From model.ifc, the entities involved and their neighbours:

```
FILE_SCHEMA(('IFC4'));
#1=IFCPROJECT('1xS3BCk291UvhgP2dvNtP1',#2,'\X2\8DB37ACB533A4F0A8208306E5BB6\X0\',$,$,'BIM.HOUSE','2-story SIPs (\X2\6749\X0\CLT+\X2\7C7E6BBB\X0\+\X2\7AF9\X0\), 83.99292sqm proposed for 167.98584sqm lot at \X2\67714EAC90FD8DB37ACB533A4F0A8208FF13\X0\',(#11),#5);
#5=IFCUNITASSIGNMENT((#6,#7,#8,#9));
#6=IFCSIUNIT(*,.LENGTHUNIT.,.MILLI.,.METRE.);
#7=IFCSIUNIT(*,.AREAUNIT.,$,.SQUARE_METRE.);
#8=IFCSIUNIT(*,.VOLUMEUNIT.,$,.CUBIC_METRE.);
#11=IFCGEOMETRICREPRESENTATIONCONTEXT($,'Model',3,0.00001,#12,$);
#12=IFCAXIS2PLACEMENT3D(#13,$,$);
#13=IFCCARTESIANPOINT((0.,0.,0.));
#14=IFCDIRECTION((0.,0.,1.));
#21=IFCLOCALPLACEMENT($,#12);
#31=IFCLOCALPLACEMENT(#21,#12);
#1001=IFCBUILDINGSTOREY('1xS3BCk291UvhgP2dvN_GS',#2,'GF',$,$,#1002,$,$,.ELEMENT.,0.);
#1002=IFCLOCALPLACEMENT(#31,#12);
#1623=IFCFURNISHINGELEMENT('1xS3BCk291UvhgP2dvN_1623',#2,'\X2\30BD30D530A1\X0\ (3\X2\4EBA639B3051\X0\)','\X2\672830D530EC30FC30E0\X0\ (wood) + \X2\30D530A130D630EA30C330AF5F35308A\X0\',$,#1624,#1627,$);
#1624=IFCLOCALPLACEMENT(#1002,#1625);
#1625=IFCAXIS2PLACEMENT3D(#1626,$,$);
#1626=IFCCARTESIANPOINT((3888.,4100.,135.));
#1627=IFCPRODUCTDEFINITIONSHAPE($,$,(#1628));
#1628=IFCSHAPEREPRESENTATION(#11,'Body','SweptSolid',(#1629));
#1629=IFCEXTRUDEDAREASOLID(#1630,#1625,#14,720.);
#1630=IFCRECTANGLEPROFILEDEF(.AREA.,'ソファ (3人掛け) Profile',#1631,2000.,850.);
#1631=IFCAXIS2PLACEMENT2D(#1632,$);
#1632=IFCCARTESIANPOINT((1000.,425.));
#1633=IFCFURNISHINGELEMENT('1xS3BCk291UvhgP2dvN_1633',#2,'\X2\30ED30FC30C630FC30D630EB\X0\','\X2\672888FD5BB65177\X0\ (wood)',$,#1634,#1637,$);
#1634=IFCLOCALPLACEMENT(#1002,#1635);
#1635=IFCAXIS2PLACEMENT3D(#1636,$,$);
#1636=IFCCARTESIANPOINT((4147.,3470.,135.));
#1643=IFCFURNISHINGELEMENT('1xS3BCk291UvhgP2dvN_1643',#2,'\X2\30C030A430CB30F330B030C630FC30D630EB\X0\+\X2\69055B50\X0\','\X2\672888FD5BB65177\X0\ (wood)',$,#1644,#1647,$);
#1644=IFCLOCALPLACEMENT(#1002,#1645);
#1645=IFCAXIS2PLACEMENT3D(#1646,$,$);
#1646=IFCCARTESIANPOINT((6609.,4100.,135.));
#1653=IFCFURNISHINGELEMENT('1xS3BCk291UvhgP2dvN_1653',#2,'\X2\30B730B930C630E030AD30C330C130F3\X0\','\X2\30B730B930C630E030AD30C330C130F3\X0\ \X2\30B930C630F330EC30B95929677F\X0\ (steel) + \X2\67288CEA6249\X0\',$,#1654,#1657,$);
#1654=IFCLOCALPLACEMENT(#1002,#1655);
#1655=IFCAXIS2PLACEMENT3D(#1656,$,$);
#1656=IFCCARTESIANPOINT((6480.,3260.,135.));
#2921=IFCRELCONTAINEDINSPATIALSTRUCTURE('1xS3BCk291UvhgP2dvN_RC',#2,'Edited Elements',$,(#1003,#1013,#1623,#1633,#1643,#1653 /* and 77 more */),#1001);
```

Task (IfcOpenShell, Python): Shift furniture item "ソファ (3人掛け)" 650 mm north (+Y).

```python
import ifcopenshell
import ifcopenshell.api.geometry
import ifcopenshell.util.placement
import ifcopenshell.util.unit

model = ifcopenshell.open("model.ifc")
unit_scale = ifcopenshell.util.unit.calculate_unit_scale(model)

item = model.by_guid("1xS3BCk291UvhgP2dvN_1623")
matrix = ifcopenshell.util.placement.get_local_placement(item.ObjectPlacement)
matrix[1, 3] += 0.65 / unit_scale
ifcopenshell.api.geometry.edit_object_placement(model, product=item, matrix=matrix, is_si=False)

print(ifcopenshell.util.placement.get_local_placement(item.ObjectPlacement).round(3) + 0.0)

model.write("model_v2.ifc")
```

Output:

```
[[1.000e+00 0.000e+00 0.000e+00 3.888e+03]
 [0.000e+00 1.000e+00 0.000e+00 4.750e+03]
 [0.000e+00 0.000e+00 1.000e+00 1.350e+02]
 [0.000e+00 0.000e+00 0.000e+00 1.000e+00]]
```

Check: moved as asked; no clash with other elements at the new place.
